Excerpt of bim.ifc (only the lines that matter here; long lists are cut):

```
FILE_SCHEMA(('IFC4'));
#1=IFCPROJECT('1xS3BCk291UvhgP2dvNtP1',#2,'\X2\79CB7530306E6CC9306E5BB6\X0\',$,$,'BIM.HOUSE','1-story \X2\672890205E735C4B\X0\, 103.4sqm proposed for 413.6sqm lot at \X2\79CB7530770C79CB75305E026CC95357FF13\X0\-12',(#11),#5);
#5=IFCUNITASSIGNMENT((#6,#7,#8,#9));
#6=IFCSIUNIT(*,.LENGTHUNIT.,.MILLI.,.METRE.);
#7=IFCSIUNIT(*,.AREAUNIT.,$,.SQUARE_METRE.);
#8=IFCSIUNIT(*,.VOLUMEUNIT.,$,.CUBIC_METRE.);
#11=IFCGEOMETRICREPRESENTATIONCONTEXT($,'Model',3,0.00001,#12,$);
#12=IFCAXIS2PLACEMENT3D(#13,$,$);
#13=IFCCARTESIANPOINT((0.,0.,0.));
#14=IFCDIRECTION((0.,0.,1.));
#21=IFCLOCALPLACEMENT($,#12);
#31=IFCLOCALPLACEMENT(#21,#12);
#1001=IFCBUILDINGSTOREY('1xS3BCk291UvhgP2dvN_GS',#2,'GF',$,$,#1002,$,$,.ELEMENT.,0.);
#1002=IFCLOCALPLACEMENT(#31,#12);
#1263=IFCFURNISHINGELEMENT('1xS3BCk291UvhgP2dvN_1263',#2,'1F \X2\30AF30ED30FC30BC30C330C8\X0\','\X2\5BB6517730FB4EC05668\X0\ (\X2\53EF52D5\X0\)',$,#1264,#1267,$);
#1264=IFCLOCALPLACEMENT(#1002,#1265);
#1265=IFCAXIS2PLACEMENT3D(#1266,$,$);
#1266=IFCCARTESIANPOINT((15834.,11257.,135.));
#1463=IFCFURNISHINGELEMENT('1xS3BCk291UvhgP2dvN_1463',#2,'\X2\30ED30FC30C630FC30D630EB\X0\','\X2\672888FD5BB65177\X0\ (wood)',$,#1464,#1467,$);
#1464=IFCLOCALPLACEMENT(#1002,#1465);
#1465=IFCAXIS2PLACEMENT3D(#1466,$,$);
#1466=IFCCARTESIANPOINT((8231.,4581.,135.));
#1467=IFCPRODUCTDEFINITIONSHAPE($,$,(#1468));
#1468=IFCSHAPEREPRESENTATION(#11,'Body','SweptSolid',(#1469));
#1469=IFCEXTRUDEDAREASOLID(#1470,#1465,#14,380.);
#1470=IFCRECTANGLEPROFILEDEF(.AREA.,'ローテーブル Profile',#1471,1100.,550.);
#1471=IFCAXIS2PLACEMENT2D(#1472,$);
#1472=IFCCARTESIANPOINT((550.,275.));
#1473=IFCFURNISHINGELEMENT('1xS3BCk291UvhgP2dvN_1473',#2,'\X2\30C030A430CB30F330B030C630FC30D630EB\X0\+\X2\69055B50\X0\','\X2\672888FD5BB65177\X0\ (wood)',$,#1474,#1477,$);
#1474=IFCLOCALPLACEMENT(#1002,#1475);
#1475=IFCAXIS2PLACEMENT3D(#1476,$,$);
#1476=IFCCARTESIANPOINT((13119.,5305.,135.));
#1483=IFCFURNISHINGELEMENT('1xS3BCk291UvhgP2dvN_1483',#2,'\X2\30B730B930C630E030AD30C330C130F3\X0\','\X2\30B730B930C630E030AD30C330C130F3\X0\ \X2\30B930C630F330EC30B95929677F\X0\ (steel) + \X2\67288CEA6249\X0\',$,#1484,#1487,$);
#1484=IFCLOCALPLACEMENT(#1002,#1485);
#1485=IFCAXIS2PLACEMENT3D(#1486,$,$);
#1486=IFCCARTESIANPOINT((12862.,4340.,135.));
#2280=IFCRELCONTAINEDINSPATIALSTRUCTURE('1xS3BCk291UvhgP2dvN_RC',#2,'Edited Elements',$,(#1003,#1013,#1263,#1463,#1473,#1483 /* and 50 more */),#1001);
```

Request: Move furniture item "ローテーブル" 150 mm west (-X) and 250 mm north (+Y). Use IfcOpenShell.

```python
import ifcopenshell
import ifcopenshell.api.geometry
import ifcopenshell.util.placement
import ifcopenshell.util.unit

model = ifcopenshell.open("bim.ifc")
unit_scale = ifcopenshell.util.unit.calculate_unit_scale(model)

item = model.by_guid("1xS3BCk291UvhgP2dvN_1463")
matrix = ifcopenshell.util.placement.get_local_placement(item.ObjectPlacement)
matrix[0, 3] -= 0.15 / unit_scale
matrix[1, 3] += 0.25 / unit_scale
ifcopenshell.api.geometry.edit_object_placement(model, product=item, matrix=matrix, is_si=False)

print(ifcopenshell.util.placement.get_local_placement(item.ObjectPlacement).round(3) + 0.0)

model.write("bim_v2.ifc")
```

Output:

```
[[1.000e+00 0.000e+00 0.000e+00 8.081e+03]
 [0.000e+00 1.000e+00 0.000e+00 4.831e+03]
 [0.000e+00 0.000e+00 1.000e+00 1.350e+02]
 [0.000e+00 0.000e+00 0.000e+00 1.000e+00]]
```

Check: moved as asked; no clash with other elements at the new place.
